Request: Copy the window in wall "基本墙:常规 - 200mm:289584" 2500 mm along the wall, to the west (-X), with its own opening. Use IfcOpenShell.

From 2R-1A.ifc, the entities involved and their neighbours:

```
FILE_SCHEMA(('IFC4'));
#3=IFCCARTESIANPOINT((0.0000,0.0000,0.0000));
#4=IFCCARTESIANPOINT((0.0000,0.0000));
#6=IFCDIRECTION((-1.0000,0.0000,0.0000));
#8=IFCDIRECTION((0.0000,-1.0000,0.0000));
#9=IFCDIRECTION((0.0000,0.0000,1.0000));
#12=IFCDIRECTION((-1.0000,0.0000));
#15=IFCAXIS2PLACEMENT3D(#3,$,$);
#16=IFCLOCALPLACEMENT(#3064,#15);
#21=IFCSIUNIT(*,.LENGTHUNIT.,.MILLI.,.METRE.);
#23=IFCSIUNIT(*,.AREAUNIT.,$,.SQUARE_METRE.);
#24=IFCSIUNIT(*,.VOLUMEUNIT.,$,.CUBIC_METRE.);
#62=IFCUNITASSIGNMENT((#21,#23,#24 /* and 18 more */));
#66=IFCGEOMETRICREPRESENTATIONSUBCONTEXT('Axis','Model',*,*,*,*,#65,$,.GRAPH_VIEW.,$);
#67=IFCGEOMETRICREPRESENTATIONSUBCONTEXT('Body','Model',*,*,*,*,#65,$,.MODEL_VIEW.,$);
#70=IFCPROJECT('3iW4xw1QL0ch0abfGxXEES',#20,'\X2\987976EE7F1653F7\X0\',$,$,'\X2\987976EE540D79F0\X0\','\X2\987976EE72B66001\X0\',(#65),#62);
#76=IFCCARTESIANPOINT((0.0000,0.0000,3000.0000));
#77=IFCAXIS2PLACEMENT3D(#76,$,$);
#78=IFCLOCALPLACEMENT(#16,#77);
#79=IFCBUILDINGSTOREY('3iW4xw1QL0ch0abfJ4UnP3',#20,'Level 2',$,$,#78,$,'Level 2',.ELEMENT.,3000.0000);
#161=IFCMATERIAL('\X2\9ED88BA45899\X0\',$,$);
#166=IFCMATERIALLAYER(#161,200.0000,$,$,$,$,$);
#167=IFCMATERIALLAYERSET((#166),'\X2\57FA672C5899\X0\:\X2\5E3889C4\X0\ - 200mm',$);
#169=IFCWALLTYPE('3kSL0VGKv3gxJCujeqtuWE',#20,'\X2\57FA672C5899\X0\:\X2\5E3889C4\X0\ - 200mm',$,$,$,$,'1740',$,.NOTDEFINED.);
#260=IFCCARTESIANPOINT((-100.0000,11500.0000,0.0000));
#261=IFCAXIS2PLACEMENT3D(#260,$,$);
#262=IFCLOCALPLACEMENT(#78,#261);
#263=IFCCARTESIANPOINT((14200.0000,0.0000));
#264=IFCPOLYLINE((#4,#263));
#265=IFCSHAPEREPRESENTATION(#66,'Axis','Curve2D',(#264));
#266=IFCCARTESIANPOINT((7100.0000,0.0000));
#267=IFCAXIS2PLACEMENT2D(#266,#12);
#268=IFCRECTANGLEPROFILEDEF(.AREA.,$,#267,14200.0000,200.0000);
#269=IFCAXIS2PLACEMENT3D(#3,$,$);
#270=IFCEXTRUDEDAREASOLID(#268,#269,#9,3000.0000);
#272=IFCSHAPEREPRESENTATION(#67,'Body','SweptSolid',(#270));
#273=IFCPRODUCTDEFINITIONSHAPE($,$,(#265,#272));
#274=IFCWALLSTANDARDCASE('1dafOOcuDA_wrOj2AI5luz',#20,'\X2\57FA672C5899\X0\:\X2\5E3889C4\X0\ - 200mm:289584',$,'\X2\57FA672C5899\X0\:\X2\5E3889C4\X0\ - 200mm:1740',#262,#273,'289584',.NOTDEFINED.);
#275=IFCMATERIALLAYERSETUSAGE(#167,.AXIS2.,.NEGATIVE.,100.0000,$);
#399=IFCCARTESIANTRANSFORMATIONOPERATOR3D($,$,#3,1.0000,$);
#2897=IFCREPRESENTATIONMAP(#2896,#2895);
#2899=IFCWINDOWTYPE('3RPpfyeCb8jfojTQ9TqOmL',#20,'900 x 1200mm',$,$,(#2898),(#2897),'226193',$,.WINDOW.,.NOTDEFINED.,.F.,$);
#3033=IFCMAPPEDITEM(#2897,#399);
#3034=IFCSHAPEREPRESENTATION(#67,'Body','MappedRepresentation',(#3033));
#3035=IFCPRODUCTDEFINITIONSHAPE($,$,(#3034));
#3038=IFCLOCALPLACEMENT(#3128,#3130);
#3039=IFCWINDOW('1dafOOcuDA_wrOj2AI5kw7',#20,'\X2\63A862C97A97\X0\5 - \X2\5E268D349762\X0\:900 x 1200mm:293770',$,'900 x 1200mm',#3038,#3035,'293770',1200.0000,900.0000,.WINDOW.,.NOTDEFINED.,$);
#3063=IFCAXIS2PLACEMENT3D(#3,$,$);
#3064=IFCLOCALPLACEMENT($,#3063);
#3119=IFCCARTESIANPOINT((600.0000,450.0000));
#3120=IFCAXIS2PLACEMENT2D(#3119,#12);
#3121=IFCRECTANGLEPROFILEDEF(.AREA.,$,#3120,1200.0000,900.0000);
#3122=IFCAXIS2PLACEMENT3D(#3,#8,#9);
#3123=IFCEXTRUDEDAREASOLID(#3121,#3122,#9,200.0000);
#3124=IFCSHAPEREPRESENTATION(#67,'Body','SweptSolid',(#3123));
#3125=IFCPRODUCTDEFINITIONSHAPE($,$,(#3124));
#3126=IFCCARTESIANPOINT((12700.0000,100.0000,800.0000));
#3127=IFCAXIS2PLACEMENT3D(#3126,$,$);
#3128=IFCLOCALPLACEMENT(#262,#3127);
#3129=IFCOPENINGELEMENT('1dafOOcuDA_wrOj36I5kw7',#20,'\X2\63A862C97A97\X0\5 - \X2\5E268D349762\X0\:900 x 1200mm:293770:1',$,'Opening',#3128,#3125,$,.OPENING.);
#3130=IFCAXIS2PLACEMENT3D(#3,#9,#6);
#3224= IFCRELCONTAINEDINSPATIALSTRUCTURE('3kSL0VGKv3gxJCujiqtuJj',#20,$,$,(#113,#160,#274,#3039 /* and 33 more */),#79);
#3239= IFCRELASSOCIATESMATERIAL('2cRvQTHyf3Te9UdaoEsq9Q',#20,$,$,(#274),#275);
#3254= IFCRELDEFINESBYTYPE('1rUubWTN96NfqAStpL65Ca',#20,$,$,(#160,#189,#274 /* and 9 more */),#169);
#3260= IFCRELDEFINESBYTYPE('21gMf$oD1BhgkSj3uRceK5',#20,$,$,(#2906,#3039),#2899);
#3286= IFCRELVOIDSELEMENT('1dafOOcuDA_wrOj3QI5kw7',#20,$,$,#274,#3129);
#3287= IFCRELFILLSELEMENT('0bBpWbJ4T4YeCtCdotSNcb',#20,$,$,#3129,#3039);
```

```python
import ifcopenshell
import ifcopenshell.api.feature
import ifcopenshell.api.geometry
import ifcopenshell.api.root
import ifcopenshell.geom
import ifcopenshell.util.element
import ifcopenshell.util.placement
import ifcopenshell.util.shape

model = ifcopenshell.open("2R-1A.ifc")
settings = ifcopenshell.geom.settings()


def volume(element):
    """Net volume in cubic metres, openings subtracted."""
    shape = ifcopenshell.geom.create_shape(settings, element)
    return ifcopenshell.util.shape.get_volume(shape.geometry)


def reuse_history(source, copy):
    """copy_class also copies each property set's owner history, people and application; keep the originals."""
    for rel in copy.IsDefinedBy:
        if rel.is_a("IfcRelDefinesByProperties") and (history := rel.RelatingPropertyDefinition.OwnerHistory):
            rel.RelatingPropertyDefinition.OwnerHistory = source.OwnerHistory
            ifcopenshell.util.element.remove_deep2(model, history)


window = model.by_guid("1dafOOcuDA_wrOj2AI5kw7")
opening = window.FillsVoids[0].RelatingOpeningElement
wall = opening.VoidsElements[0].RelatingBuildingElement
before = volume(wall)
shift = ifcopenshell.util.placement.get_local_placement(wall.ObjectPlacement)[:3, 0] * -2500.0

# copy_class copies the void relationship, type, container and properties, but no geometry.
new_opening = ifcopenshell.api.root.copy_class(model, product=opening)
new_opening.Representation = ifcopenshell.util.element.copy_deep(
    model, opening.Representation, exclude=["IfcGeometricRepresentationContext", "IfcRepresentationMap"]
)
new_opening.Name = "推拉窗5 - 带贴面:900 x 1200mm"
new_window = ifcopenshell.api.root.copy_class(model, product=window)
new_window.Representation = ifcopenshell.util.element.copy_deep(
    model, window.Representation, exclude=["IfcGeometricRepresentationContext", "IfcRepresentationMap"]
)
new_window.Name = "推拉窗5 - 带贴面:900 x 1200mm"
new_window.Tag = None
reuse_history(window, new_window)
ifcopenshell.api.feature.add_filling(model, opening=new_opening, element=new_window)

for old, new in ((opening, new_opening), (window, new_window)):
    matrix = ifcopenshell.util.placement.get_local_placement(old.ObjectPlacement)
    matrix[:3, 3] += shift
    ifcopenshell.api.geometry.edit_object_placement(model, product=new, matrix=matrix, is_si=False)

after = volume(wall)

print(f"wall volume {before:.3f} -> {after:.3f} m3")

model.write("2R-1A_edited.ifc")
```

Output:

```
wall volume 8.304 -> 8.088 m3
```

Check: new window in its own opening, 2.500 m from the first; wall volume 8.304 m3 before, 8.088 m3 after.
